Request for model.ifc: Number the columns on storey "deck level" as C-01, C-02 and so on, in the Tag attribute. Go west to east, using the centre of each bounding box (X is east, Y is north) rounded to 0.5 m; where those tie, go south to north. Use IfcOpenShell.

First a look at what the model holds.

```python
import ifcopenshell
import ifcopenshell.util.element
import ifcopenshell.util.placement

model = ifcopenshell.open("model.ifc")
print(model.schema)
storey = next(s for s in model.by_type("IfcBuildingStorey") if s.Name == "deck level")
columns = [e for e in ifcopenshell.util.element.get_decomposition(storey) if e.is_a("IfcColumn")]
for e in sorted(columns, key=lambda e: e.id()):
    origin = ifcopenshell.util.placement.get_local_placement(e.ObjectPlacement)[:3, 3]
    print(e.id(), e.Tag, e.Name, origin.round(2) + 0.0, sep=" | ")
```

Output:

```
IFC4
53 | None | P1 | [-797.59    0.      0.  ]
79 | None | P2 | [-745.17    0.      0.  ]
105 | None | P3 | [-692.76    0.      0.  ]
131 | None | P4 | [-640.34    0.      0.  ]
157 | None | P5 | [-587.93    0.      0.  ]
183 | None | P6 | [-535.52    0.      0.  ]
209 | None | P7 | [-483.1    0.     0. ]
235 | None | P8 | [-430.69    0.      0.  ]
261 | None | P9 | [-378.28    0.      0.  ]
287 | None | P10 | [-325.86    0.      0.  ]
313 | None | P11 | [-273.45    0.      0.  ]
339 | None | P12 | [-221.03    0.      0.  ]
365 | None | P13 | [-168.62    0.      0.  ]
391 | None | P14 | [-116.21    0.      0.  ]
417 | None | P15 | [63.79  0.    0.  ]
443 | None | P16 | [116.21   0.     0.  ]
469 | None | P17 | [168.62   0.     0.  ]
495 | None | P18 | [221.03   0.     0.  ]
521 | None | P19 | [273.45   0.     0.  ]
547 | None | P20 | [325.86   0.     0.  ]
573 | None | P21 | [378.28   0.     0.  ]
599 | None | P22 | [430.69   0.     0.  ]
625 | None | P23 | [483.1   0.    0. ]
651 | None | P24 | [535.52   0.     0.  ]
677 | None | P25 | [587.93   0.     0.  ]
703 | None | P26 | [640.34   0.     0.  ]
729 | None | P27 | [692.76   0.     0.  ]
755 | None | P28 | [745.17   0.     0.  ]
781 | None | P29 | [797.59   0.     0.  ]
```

```python
import ifcopenshell
import ifcopenshell.geom
import ifcopenshell.util.element
import ifcopenshell.util.shape

model = ifcopenshell.open("model.ifc")
settings = ifcopenshell.geom.settings()
settings.set("use-world-coords", True)


def centre(element):
    shape = ifcopenshell.geom.create_shape(settings, element)
    return ifcopenshell.util.shape.get_bbox_centroid(shape.geometry)


storey = next(s for s in model.by_type("IfcBuildingStorey") if s.Name == "deck level")
columns = [e for e in ifcopenshell.util.element.get_decomposition(storey) if e.is_a("IfcColumn")]

# Insertion points can sit at a corner or the storey origin, so sort by the geometry (in metres).
centres = {e: centre(e) for e in columns}
columns.sort(key=lambda e: (round(centres[e][0] / 0.5), centres[e][1]))

for i, e in enumerate(columns, start=1):
    number = f"C-{i:02d}"
    e.Tag = number
    print(e.id(), number)

model.write("model_edited.ifc")
```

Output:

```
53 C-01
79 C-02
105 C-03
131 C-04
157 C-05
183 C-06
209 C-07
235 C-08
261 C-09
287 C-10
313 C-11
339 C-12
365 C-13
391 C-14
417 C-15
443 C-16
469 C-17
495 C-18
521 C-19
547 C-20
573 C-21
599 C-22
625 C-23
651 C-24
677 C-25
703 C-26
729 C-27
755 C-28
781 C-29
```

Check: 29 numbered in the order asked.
